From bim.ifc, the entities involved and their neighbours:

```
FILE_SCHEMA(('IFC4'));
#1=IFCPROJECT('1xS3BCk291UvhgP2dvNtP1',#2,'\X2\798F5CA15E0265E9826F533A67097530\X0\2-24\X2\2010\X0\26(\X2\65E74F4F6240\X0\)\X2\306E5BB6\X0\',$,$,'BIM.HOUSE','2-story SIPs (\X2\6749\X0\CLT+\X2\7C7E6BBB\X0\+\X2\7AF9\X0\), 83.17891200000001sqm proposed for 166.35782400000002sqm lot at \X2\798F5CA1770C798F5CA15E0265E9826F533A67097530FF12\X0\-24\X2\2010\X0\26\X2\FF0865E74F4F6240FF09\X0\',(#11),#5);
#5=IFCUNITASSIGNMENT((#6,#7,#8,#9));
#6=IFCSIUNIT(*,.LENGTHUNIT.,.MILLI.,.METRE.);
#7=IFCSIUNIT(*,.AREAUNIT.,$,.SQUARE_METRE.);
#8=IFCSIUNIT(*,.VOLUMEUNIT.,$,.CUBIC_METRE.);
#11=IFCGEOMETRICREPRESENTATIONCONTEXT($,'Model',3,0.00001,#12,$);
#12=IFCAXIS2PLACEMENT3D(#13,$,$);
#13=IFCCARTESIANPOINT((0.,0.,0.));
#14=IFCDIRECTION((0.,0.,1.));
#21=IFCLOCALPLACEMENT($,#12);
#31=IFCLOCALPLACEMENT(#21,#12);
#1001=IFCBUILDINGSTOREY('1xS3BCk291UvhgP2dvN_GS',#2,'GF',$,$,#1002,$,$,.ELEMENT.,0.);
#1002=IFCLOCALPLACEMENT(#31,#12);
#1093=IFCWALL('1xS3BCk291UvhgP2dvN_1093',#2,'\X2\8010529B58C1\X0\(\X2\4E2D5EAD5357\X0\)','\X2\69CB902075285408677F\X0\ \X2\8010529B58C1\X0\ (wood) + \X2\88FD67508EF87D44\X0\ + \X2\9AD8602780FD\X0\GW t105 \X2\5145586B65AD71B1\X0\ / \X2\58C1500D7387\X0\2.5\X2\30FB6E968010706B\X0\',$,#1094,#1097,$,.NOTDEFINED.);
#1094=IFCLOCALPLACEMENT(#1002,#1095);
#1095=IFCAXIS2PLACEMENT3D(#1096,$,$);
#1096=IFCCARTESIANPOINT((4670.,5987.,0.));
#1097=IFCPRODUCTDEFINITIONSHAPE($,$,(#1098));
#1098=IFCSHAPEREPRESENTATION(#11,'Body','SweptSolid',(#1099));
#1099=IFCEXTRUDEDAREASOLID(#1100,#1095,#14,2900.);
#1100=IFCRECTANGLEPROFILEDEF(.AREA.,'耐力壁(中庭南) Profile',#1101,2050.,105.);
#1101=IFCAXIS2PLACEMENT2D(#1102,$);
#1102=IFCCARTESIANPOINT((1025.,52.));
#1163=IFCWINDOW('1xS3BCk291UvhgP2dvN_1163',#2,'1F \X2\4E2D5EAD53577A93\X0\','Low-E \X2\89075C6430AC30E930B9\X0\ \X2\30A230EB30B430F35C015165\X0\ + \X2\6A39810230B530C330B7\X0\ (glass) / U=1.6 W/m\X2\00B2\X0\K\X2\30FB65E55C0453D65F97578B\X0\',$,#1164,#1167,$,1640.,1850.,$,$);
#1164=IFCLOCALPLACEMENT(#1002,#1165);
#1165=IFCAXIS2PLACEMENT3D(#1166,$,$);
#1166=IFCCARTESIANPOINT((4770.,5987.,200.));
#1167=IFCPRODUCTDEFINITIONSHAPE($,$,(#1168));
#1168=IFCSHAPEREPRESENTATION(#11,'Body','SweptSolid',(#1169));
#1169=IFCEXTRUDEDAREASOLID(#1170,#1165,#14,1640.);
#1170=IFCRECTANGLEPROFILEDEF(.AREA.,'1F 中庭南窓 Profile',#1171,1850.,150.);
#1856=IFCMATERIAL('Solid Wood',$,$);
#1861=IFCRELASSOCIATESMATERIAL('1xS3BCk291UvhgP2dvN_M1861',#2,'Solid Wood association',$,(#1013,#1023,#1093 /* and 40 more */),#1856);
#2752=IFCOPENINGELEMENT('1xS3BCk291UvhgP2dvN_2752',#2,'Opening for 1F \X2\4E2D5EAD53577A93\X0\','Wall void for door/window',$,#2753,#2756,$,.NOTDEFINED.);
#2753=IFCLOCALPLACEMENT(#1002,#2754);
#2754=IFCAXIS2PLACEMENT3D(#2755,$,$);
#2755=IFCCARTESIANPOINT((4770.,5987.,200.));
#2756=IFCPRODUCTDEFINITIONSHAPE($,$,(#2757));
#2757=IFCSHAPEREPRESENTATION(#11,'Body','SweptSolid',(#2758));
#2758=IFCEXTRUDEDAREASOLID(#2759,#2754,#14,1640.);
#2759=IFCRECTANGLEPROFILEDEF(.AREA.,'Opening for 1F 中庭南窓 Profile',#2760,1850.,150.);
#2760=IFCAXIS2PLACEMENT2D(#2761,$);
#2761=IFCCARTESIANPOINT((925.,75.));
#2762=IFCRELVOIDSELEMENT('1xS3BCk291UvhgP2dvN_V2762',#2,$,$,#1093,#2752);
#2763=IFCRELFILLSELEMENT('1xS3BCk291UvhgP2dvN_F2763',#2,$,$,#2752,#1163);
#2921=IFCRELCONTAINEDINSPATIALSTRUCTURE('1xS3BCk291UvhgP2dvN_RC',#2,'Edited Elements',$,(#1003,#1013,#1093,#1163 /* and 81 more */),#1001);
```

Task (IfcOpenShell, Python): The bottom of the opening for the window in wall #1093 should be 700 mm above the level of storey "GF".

```python
import numpy as np
import ifcopenshell
import ifcopenshell.api.geometry
import ifcopenshell.geom
import ifcopenshell.util.element
import ifcopenshell.util.placement
import ifcopenshell.util.shape
import ifcopenshell.util.unit

model = ifcopenshell.open("bim.ifc")
unit_scale = ifcopenshell.util.unit.calculate_unit_scale(model)

window = model.by_guid("1xS3BCk291UvhgP2dvN_1163")
opening = window.FillsVoids[0].RelatingOpeningElement
storey = ifcopenshell.util.element.get_container(window, ifc_class="IfcBuildingStorey")
level = ifcopenshell.util.placement.get_local_placement(storey.ObjectPlacement)[2, 3]

# The opening's origin need not be at the sill, so measure its lowest point.
shape = ifcopenshell.geom.create_shape(ifcopenshell.geom.settings(), opening)
bottom = ifcopenshell.util.shape.get_shape_bottom_elevation(shape, shape.geometry) / unit_scale
dz = level + 0.7 / unit_scale - bottom

shift = np.array([0.0, 0.0, dz])
# The window is not placed relative to its opening, so move both.
for product in (opening, window):
    matrix = ifcopenshell.util.placement.get_local_placement(product.ObjectPlacement)
    matrix[:3, 3] += shift
    ifcopenshell.api.geometry.edit_object_placement(model, product=product, matrix=matrix, is_si=False)

print(f"moved by {dz * unit_scale:+.3f} m")

model.write("bim-out.ifc")
```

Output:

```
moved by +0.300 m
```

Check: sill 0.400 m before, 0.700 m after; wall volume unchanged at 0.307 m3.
